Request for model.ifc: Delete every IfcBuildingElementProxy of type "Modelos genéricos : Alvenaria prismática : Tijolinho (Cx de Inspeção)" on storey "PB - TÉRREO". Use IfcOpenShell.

First a look at what the model holds.

```python
import ifcopenshell
import ifcopenshell.util.element

model = ifcopenshell.open("model.ifc")
print(model.schema)
storey = next(s for s in model.by_type("IfcBuildingStorey") if s.Name == "PB - TÉRREO")
proxies = [e for e in ifcopenshell.util.element.get_decomposition(storey) if e.is_a("IfcBuildingElementProxy")]
seen = {}
for e in proxies:
    element_type = ifcopenshell.util.element.get_type(e)
    name = element_type.Name if element_type not in (None, e) else None
    seen[name] = seen.get(name, 0) + 1
for name, count in sorted(seen.items(), key=str):
    print(count, "x", name)
```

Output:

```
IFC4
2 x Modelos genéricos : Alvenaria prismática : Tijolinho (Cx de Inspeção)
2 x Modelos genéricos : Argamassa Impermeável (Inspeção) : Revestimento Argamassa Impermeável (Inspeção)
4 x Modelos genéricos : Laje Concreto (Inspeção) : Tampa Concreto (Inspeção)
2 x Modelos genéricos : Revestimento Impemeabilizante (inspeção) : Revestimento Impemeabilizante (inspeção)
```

```python
import ifcopenshell
import ifcopenshell.api.root
import ifcopenshell.util.element

model = ifcopenshell.open("model.ifc")

storey = next(s for s in model.by_type("IfcBuildingStorey") if s.Name == "PB - TÉRREO")
proxies = [e for e in ifcopenshell.util.element.get_decomposition(storey) if e.is_a("IfcBuildingElementProxy")]
targets = [e for e in proxies if (t := ifcopenshell.util.element.get_type(e)) not in (None, e) and t.Name == "Modelos genéricos : Alvenaria prismática : Tijolinho (Cx de Inspeção)"]

for e in targets:
    ifcopenshell.api.root.remove_product(model, product=e)
print(len(targets), "removed")

model.write("model-out.ifc")
```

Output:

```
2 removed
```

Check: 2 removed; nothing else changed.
